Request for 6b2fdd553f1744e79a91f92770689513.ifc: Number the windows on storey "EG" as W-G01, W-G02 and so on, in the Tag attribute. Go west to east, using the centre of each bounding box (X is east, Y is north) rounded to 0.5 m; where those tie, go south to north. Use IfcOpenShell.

First a look at what the model holds.

```python
import ifcopenshell
import ifcopenshell.util.element
import ifcopenshell.util.placement

model = ifcopenshell.open("6b2fdd553f1744e79a91f92770689513.ifc")
print(model.schema)
storey = next(s for s in model.by_type("IfcBuildingStorey") if s.Name == "EG")
windows = [e for e in ifcopenshell.util.element.get_decomposition(storey) if e.is_a("IfcWindow")]
for e in sorted(windows, key=lambda e: e.id()):
    origin = ifcopenshell.util.placement.get_local_placement(e.ObjectPlacement)[:3, 3]
    print(e.id(), e.Tag, e.Name, origin.round(2) + 0.0, sep=" | ")
```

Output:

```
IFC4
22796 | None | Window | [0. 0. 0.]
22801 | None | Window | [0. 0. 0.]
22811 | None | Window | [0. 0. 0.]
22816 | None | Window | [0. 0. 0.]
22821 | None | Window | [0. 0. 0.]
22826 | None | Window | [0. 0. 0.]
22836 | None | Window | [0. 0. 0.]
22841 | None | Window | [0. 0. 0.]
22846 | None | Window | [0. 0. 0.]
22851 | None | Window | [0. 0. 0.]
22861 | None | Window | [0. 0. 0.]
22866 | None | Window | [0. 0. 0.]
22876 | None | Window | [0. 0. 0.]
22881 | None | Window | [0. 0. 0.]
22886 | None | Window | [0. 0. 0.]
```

```python
import ifcopenshell
import ifcopenshell.geom
import ifcopenshell.util.element
import ifcopenshell.util.shape

model = ifcopenshell.open("6b2fdd553f1744e79a91f92770689513.ifc")
settings = ifcopenshell.geom.settings()
settings.set("use-world-coords", True)


def centre(element):
    shape = ifcopenshell.geom.create_shape(settings, element)
    return ifcopenshell.util.shape.get_bbox_centroid(shape.geometry)


storey = next(s for s in model.by_type("IfcBuildingStorey") if s.Name == "EG")
windows = [e for e in ifcopenshell.util.element.get_decomposition(storey) if e.is_a("IfcWindow")]

# Insertion points can sit at a corner or the storey origin, so sort by the geometry (in metres).
centres = {e: centre(e) for e in windows}
windows.sort(key=lambda e: (round(centres[e][0] / 0.5), centres[e][1]))

for i, e in enumerate(windows, start=1):
    number = f"W-G{i:02d}"
    e.Tag = number
    print(e.id(), number)

model.write("6b2fdd553f1744e79a91f92770689513-out.ifc")
```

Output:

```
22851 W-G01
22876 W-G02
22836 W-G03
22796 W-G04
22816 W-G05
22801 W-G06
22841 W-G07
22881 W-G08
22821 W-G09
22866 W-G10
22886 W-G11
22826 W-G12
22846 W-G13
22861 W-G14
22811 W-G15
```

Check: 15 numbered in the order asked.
